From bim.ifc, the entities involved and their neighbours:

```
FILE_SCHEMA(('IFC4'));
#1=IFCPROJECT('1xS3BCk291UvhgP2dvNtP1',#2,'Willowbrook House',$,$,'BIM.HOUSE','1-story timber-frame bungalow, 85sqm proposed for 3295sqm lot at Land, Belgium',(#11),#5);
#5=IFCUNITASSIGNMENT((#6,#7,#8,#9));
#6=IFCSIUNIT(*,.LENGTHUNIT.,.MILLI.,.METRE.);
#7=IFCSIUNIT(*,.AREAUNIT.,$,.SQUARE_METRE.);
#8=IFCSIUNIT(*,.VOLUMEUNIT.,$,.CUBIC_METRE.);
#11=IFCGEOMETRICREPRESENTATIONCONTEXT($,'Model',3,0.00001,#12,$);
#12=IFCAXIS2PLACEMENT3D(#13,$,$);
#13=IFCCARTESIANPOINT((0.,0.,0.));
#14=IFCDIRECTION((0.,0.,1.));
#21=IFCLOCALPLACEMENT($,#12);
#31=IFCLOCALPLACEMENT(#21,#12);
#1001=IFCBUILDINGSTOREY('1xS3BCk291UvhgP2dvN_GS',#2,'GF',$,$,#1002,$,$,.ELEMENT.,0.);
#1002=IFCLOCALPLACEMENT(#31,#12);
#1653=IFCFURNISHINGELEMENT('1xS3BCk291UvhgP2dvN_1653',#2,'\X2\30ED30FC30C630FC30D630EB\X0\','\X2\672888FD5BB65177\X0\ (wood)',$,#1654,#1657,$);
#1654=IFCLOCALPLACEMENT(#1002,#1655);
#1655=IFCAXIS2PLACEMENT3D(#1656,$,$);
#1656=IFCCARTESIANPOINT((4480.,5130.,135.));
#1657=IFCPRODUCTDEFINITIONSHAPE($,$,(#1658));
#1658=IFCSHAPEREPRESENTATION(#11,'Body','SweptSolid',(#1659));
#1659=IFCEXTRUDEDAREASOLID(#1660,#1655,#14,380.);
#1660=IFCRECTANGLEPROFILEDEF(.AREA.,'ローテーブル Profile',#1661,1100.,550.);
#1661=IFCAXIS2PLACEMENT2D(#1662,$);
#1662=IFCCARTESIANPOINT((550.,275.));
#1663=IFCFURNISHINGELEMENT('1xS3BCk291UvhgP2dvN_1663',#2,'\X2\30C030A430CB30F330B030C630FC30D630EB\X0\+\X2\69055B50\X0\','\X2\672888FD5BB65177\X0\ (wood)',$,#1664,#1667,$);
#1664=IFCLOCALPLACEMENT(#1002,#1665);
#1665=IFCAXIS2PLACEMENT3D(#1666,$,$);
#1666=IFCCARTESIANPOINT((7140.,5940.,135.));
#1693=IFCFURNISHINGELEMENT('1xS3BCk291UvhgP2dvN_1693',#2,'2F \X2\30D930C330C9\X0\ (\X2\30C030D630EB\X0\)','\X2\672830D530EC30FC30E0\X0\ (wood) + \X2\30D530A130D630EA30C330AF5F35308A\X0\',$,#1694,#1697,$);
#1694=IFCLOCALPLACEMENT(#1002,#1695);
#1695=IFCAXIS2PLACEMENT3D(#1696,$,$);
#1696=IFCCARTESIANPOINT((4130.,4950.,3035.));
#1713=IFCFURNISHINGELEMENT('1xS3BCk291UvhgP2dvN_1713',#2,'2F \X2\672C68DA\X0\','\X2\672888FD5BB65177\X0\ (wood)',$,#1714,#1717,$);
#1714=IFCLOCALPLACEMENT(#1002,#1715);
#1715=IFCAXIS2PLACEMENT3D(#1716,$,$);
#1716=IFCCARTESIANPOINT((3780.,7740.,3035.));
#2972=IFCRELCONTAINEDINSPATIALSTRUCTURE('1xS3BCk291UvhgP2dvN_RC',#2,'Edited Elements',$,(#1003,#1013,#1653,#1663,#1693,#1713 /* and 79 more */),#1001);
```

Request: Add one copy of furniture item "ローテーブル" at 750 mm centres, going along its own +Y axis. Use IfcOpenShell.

```python
import ifcopenshell
import ifcopenshell.api.geometry
import ifcopenshell.api.root
import ifcopenshell.util.element
import ifcopenshell.util.placement
import ifcopenshell.util.unit

model = ifcopenshell.open("bim.ifc")
unit_scale = ifcopenshell.util.unit.calculate_unit_scale(model)


def reuse_history(source, copy):
    """copy_class also copies each property set's owner history, people and application; keep the originals."""
    for rel in copy.IsDefinedBy:
        if rel.is_a("IfcRelDefinesByProperties") and (history := rel.RelatingPropertyDefinition.OwnerHistory):
            rel.RelatingPropertyDefinition.OwnerHistory = source.OwnerHistory
            ifcopenshell.util.element.remove_deep2(model, history)


source = model.by_guid("1xS3BCk291UvhgP2dvN_1653")
base = ifcopenshell.util.placement.get_local_placement(source.ObjectPlacement)
step = base[:3, 1] * 0.75 / unit_scale

for i in range(1, 2):
    copy = ifcopenshell.api.root.copy_class(model, product=source)
    copy.Representation = ifcopenshell.util.element.copy_deep(
        model, source.Representation, exclude=["IfcGeometricRepresentationContext", "IfcRepresentationMap"]
    )
    reuse_history(source, copy)
    matrix = base.copy()
    matrix[:3, 3] += i * step
    print("added at", matrix[:3, 3].round(3) + 0.0)
    ifcopenshell.api.geometry.edit_object_placement(model, product=copy, matrix=matrix, is_si=False)

model.write("bim_edited.ifc")
```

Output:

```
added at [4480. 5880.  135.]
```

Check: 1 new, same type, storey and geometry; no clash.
